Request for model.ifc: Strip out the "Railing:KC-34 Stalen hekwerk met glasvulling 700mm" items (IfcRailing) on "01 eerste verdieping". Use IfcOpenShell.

First a look at what the model holds.

```python
import ifcopenshell
import ifcopenshell.util.element

model = ifcopenshell.open("model.ifc")
print(model.schema)
storey = next(s for s in model.by_type("IfcBuildingStorey") if s.Name == "01 eerste verdieping")
railings = [e for e in ifcopenshell.util.element.get_decomposition(storey) if e.is_a("IfcRailing")]
seen = {}
for e in railings:
    element_type = ifcopenshell.util.element.get_type(e)
    name = element_type.Name if element_type not in (None, e) else None
    seen[name] = seen.get(name, 0) + 1
for name, count in sorted(seen.items(), key=str):
    print(count, "x", name)
```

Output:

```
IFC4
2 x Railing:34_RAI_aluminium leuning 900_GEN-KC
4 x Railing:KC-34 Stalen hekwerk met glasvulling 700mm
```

```python
import ifcopenshell
import ifcopenshell.api.root
import ifcopenshell.util.element

model = ifcopenshell.open("model.ifc")

storey = next(s for s in model.by_type("IfcBuildingStorey") if s.Name == "01 eerste verdieping")
railings = [e for e in ifcopenshell.util.element.get_decomposition(storey) if e.is_a("IfcRailing")]
targets = [e for e in railings if (t := ifcopenshell.util.element.get_type(e)) not in (None, e) and t.Name == "Railing:KC-34 Stalen hekwerk met glasvulling 700mm"]

for e in targets:
    ifcopenshell.api.root.remove_product(model, product=e)
print(len(targets), "removed")

model.write("model-out.ifc")
```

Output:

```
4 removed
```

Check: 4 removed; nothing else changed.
